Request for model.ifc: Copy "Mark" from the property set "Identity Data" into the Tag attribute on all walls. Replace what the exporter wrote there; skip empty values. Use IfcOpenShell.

First a look at what the model holds.

```python
import ifcopenshell
import ifcopenshell.util.element

model = ifcopenshell.open("model.ifc")
print(model.schema)
walls = model.by_type("IfcWall")
print(len(walls), "walls")
for e in walls[:8]:
    source = ifcopenshell.util.element.get_pset(e, "Identity Data", "Mark")
    target = e.Tag
    print(e.id(), repr(source), repr(target), sep=" | ")
```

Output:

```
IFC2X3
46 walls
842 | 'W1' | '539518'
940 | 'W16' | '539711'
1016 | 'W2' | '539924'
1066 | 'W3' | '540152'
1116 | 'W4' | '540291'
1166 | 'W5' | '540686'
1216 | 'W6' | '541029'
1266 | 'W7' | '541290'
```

```python
import ifcopenshell
import ifcopenshell.util.element

model = ifcopenshell.open("model.ifc")

count = 0
for e in model.by_type("IfcWall"):
    value = ifcopenshell.util.element.get_pset(e, "Identity Data", "Mark")
    current = e.Tag
    if not value or not value.strip() or current == value:
        continue
    e.Tag = value
    count += 1

print(count, "walls updated")

model.write("model_updated.ifc")
```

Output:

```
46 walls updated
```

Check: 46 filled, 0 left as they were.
